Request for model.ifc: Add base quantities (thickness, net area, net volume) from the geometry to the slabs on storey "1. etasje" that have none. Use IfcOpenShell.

First a look at what the model holds.

```python
import ifcopenshell
import ifcopenshell.util.element
import ifcopenshell.util.unit

model = ifcopenshell.open("model.ifc")
print(model.schema)
for unit_type in ("LENGTHUNIT", "AREAUNIT", "VOLUMEUNIT"):
    print(unit_type, ifcopenshell.util.unit.calculate_unit_scale(model, unit_type))
storey = next(s for s in model.by_type("IfcBuildingStorey") if s.Name == "1. etasje")
slabs = [e for e in ifcopenshell.util.element.get_decomposition(storey) if e.is_a("IfcSlab")]
for e in sorted(slabs, key=lambda e: e.id()):
    print(e.id(), e.is_a(), e.Name, list(ifcopenshell.util.element.get_psets(e, qtos_only=True)), sep=" | ")
```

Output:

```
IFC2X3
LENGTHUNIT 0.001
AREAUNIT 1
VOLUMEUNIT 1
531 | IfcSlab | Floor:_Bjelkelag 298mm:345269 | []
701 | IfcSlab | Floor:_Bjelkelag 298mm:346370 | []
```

```python
import ifcopenshell
import ifcopenshell.api.pset
import ifcopenshell.geom
import ifcopenshell.util.element
import ifcopenshell.util.shape
import ifcopenshell.util.unit

model = ifcopenshell.open("model.ifc")
unit_scale = ifcopenshell.util.unit.calculate_unit_scale(model)
area_scale = ifcopenshell.util.unit.calculate_unit_scale(model, "AREAUNIT")
volume_scale = ifcopenshell.util.unit.calculate_unit_scale(model, "VOLUMEUNIT")
settings = ifcopenshell.geom.settings()

storey = next(s for s in model.by_type("IfcBuildingStorey") if s.Name == "1. etasje")
slabs = [e for e in ifcopenshell.util.element.get_decomposition(storey) if e.is_a("IfcSlab")]

for e in sorted(slabs, key=lambda e: e.id()):
    if ifcopenshell.util.element.get_psets(e, qtos_only=True, should_inherit=False):
        continue
    # Geometry comes back in metres, in the element's own axes.
    shape = ifcopenshell.geom.create_shape(settings, e)
    values = {
        "Width": ifcopenshell.util.shape.get_z(shape.geometry) / unit_scale,
        "NetArea": ifcopenshell.util.shape.get_footprint_area(shape.geometry) / area_scale,
        "NetVolume": ifcopenshell.util.shape.get_volume(shape.geometry) / volume_scale,
    }
    qto = ifcopenshell.api.pset.add_qto(model, product=e, name="BaseQuantities")
    ifcopenshell.api.pset.edit_qto(model, qto=qto, properties=values)
    print(e.id(), {k: round(v, 3) for k, v in values.items()})

model.write("model_edited.ifc")
```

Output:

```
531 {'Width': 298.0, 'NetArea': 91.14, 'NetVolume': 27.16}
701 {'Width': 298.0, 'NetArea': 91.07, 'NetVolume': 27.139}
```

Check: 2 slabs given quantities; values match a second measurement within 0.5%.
